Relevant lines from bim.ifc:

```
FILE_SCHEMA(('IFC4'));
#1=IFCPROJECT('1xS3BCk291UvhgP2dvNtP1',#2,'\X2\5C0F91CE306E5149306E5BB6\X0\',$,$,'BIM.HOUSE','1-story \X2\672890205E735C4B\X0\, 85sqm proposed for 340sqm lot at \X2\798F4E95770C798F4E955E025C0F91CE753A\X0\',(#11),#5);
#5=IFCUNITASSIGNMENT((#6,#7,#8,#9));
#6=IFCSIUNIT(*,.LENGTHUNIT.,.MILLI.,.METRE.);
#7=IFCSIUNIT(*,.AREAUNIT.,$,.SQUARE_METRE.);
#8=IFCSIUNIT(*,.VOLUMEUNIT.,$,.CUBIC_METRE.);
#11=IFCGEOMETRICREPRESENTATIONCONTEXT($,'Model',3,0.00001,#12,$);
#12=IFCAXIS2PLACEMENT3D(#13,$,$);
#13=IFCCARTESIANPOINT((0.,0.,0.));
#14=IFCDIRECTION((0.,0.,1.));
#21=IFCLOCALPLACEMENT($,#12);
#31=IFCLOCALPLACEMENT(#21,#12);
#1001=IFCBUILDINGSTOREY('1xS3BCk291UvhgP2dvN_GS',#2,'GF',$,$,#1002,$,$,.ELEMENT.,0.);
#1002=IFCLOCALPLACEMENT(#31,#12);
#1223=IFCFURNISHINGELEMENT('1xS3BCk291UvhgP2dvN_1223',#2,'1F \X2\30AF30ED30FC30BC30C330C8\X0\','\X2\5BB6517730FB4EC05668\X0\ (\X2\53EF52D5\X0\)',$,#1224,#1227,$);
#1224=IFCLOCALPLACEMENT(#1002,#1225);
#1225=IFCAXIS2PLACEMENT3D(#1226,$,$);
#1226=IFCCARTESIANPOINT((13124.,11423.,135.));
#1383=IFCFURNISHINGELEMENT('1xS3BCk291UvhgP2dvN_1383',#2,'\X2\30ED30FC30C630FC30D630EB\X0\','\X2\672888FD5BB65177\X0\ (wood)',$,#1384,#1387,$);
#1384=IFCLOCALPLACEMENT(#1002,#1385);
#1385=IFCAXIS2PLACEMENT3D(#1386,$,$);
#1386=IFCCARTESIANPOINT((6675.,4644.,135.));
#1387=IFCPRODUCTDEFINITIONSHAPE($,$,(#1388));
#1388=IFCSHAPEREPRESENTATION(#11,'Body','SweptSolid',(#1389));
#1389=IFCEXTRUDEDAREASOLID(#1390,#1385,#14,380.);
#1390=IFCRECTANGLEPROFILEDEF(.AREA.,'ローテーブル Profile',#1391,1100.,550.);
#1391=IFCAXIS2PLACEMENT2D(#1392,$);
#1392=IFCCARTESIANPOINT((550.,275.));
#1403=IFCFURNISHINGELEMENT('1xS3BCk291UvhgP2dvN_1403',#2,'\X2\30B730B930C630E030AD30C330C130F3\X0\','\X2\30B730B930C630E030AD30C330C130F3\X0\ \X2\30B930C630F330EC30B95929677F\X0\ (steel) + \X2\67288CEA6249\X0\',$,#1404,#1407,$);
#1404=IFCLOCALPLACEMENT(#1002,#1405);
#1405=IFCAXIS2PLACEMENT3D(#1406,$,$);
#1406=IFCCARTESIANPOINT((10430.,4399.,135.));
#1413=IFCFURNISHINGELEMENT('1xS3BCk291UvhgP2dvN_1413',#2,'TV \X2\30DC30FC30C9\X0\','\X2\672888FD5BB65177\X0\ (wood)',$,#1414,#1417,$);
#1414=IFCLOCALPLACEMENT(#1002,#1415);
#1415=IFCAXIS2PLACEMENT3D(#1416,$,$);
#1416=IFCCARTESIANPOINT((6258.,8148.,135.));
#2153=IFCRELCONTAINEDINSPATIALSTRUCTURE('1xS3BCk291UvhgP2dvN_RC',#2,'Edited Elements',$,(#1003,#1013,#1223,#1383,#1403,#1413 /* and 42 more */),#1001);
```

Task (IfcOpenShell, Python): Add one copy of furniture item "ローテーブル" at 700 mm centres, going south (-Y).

```python
import numpy as np
import ifcopenshell
import ifcopenshell.api.geometry
import ifcopenshell.api.root
import ifcopenshell.util.element
import ifcopenshell.util.placement

model = ifcopenshell.open("bim.ifc")


def reuse_history(source, copy):
    """copy_class also copies each property set's owner history, people and application; keep the originals."""
    for rel in copy.IsDefinedBy:
        if rel.is_a("IfcRelDefinesByProperties") and (history := rel.RelatingPropertyDefinition.OwnerHistory):
            rel.RelatingPropertyDefinition.OwnerHistory = source.OwnerHistory
            ifcopenshell.util.element.remove_deep2(model, history)


source = model.by_guid("1xS3BCk291UvhgP2dvN_1383")
base = ifcopenshell.util.placement.get_local_placement(source.ObjectPlacement)
step = np.array([0.0, -1.0, 0.0]) * 700.0

for i in range(1, 2):
    copy = ifcopenshell.api.root.copy_class(model, product=source)
    copy.Representation = ifcopenshell.util.element.copy_deep(
        model, source.Representation, exclude=["IfcGeometricRepresentationContext", "IfcRepresentationMap"]
    )
    reuse_history(source, copy)
    matrix = base.copy()
    matrix[:3, 3] += i * step
    print("added at", matrix[:3, 3].round(3) + 0.0)
    ifcopenshell.api.geometry.edit_object_placement(model, product=copy, matrix=matrix, is_si=False)

model.write("bim_edited.ifc")
```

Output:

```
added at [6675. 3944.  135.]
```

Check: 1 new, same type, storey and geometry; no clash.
